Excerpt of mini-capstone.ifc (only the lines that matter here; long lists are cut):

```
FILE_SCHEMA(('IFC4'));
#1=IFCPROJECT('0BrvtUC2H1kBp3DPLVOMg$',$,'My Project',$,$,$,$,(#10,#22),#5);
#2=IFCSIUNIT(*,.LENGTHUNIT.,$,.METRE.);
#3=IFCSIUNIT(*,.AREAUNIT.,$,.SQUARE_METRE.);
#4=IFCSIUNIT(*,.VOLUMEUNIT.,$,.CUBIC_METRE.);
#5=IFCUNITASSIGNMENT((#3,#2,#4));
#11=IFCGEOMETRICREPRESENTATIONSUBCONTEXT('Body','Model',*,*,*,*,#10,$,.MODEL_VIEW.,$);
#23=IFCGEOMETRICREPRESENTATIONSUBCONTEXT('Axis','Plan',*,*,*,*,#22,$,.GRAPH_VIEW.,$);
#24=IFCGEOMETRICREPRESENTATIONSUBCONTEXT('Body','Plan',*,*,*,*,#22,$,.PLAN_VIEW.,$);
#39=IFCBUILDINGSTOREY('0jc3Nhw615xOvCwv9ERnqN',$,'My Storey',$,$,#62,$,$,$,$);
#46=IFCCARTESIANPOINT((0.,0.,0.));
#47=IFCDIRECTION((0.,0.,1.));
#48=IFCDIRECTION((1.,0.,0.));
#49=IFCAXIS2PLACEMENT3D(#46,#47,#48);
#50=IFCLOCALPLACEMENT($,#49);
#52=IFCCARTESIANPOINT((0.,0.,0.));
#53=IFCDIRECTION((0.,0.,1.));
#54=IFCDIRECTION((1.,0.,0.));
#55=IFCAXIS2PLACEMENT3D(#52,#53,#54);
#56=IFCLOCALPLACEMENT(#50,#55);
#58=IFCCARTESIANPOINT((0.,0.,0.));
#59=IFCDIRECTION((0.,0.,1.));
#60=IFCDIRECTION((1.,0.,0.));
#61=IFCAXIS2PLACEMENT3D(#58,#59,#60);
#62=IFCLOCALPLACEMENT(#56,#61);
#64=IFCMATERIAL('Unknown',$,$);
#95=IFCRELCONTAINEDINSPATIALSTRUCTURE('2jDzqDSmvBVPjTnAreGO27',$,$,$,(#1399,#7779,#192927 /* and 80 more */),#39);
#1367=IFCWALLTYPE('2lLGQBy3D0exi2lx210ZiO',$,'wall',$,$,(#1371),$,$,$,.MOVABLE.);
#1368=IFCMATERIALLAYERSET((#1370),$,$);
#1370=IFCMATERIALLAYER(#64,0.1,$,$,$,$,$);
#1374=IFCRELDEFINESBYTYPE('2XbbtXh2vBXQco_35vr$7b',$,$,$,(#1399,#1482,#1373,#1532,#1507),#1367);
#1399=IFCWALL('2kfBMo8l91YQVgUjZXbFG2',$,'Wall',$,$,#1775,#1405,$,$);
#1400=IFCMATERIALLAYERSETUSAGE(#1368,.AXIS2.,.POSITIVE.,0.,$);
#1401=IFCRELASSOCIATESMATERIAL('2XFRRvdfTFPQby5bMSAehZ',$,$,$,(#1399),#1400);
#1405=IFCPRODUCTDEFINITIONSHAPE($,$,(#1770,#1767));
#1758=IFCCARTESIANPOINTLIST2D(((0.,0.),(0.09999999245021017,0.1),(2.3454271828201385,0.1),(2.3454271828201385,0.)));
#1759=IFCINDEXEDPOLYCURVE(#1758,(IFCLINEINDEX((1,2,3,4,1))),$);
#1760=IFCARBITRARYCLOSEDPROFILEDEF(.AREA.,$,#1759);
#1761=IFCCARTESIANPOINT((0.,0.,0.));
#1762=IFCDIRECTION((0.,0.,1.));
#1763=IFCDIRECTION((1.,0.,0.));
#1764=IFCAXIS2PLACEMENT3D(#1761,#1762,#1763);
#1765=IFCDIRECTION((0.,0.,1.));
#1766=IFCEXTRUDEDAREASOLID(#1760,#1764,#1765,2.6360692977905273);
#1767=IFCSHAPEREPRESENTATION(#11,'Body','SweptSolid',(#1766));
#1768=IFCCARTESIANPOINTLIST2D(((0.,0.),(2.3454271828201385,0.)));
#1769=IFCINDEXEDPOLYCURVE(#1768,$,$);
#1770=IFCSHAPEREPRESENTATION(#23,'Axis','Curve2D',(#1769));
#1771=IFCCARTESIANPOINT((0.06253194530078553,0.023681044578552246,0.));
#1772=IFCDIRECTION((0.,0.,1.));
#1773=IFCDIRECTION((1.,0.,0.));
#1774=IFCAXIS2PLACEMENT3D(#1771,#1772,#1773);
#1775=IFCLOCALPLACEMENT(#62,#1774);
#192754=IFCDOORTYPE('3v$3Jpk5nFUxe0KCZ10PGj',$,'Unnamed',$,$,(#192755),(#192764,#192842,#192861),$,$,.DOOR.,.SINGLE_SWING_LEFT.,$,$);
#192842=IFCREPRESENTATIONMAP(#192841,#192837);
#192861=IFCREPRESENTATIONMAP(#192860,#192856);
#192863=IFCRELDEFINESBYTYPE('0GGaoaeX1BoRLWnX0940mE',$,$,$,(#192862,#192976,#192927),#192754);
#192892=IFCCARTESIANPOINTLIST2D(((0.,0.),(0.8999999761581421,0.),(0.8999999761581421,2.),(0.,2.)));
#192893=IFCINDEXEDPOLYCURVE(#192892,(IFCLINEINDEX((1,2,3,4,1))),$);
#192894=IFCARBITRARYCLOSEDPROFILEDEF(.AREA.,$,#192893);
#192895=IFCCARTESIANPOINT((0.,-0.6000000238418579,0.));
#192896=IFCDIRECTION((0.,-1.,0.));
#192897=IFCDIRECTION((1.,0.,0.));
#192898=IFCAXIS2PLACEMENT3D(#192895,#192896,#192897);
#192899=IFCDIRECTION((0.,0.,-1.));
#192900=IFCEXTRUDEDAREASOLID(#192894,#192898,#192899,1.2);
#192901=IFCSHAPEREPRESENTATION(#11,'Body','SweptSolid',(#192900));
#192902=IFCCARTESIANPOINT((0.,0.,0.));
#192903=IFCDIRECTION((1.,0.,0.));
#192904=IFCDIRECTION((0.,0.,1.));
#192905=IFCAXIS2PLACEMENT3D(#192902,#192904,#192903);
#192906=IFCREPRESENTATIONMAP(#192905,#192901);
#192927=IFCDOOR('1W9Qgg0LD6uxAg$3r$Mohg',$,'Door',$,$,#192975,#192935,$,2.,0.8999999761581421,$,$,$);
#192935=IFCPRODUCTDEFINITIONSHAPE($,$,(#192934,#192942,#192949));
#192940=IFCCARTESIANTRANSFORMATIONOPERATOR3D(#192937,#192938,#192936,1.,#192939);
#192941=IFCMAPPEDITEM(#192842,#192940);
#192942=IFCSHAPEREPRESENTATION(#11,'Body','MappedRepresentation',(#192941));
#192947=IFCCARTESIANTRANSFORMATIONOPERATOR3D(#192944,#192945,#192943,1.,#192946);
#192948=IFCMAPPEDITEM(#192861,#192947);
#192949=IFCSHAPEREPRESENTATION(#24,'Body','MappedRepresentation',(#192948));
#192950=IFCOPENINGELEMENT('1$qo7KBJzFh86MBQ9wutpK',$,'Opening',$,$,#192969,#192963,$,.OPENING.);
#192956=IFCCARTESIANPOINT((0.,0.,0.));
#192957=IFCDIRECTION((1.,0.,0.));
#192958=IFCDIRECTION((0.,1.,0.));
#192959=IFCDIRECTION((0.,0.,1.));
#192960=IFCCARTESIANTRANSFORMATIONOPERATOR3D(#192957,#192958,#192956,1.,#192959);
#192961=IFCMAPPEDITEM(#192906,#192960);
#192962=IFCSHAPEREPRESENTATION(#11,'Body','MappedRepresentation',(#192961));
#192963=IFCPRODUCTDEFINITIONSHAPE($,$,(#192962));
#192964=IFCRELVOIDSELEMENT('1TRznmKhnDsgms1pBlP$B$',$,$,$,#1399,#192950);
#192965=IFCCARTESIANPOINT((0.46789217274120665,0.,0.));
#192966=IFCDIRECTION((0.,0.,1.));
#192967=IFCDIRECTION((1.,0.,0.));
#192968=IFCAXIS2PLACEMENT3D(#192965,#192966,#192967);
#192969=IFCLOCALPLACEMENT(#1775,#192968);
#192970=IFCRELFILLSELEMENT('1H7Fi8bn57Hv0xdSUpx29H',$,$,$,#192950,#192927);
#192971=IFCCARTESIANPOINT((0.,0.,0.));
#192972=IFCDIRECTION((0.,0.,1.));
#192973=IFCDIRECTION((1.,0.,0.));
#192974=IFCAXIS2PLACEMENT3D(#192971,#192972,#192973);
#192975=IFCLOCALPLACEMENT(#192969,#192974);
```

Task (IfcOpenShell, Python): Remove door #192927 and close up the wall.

```python
import ifcopenshell
import ifcopenshell.api.feature
import ifcopenshell.api.root
import ifcopenshell.geom
import ifcopenshell.util.shape

model = ifcopenshell.open("mini-capstone.ifc")
settings = ifcopenshell.geom.settings()


def volume(element):
    """Net volume in cubic metres, openings subtracted."""
    shape = ifcopenshell.geom.create_shape(settings, element)
    return ifcopenshell.util.shape.get_volume(shape.geometry)


door = model.by_guid("1W9Qgg0LD6uxAg$3r$Mohg")
opening = door.FillsVoids[0].RelatingOpeningElement
wall = opening.VoidsElements[0].RelatingBuildingElement
before = volume(wall)

ifcopenshell.api.root.remove_product(model, product=door)
ifcopenshell.api.feature.remove_feature(model, feature=opening)

after = volume(wall)

print(f"wall volume {before:.3f} -> {after:.3f} m3")

model.write("mini-capstone_rev.ifc")
```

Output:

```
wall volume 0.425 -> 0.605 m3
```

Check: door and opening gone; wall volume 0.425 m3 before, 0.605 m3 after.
